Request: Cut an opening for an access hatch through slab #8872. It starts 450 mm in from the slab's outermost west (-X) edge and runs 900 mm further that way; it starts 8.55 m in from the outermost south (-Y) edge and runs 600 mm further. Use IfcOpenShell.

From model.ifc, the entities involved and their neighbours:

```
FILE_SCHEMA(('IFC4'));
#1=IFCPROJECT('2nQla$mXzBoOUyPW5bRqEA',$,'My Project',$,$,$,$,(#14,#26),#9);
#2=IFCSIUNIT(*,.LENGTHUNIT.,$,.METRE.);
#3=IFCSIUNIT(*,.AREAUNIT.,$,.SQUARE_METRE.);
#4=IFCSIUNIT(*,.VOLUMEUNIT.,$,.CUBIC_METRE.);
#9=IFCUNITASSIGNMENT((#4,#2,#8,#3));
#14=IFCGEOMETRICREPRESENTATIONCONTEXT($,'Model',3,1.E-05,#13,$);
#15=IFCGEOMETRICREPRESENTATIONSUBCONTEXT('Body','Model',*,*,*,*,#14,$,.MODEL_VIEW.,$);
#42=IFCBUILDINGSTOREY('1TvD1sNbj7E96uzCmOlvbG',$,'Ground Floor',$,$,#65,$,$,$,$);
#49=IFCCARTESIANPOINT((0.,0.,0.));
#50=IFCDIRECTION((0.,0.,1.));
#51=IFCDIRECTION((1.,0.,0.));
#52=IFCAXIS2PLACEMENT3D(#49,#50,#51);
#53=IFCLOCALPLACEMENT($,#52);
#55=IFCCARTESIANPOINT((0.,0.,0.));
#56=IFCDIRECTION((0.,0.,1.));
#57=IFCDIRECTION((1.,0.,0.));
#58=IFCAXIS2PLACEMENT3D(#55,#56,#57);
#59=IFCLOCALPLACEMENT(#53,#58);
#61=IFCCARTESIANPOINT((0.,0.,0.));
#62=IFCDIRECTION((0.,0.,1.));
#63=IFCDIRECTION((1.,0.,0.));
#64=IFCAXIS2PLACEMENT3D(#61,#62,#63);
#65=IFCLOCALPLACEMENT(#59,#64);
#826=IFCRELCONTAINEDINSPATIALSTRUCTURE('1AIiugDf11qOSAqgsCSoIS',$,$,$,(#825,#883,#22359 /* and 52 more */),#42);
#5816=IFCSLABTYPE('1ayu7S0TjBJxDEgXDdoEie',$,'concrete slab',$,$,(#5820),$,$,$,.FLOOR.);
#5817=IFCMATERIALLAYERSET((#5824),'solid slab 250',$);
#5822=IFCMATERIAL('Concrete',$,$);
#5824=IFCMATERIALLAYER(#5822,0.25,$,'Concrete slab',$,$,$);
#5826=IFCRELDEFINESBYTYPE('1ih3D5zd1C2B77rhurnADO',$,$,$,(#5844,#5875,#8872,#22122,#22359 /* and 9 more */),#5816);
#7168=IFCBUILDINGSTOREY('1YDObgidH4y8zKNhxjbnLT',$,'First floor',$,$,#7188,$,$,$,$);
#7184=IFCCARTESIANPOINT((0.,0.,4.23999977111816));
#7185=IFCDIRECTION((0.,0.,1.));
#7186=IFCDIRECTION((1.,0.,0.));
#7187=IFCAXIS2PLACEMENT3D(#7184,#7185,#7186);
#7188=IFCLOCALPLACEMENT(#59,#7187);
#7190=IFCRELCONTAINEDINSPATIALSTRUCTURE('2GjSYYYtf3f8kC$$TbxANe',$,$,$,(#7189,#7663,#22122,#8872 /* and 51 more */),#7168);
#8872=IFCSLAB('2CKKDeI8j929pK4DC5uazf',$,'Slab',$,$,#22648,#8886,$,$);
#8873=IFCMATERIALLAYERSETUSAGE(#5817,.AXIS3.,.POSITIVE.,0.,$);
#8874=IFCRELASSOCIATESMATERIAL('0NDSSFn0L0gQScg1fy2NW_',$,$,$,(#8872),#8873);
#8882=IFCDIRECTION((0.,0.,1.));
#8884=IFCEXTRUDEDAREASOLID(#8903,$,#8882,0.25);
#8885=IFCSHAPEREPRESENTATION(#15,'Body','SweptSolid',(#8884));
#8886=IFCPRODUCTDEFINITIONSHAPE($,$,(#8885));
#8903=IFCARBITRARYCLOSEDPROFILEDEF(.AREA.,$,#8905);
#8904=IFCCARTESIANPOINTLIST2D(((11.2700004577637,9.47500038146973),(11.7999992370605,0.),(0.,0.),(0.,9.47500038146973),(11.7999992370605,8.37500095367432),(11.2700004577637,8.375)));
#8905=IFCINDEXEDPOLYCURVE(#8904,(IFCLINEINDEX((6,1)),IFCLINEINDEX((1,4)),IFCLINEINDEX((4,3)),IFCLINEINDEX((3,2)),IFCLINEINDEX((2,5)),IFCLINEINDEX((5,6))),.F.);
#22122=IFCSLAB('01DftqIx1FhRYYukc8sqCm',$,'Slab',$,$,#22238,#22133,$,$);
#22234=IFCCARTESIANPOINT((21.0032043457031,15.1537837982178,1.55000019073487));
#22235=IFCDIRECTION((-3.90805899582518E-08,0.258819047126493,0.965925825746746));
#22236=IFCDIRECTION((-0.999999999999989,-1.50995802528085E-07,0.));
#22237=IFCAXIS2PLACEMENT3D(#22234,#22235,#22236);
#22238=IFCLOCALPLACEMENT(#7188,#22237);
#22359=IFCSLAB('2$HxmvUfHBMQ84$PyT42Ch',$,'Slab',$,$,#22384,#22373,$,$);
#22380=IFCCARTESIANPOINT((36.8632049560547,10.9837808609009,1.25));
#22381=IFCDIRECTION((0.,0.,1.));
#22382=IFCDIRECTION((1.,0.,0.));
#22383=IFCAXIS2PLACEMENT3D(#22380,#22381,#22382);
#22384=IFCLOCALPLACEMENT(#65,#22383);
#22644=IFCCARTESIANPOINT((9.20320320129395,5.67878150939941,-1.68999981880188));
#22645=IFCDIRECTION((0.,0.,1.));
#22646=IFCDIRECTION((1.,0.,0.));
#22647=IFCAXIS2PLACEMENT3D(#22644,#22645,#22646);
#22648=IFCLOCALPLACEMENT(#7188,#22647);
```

```python
import numpy as np
import ifcopenshell
import ifcopenshell.api.feature
import ifcopenshell.api.geometry
import ifcopenshell.api.root
import ifcopenshell.geom
import ifcopenshell.util.placement
import ifcopenshell.util.representation
import ifcopenshell.util.shape
import ifcopenshell.util.unit

model = ifcopenshell.open("model.ifc")
unit_scale = ifcopenshell.util.unit.calculate_unit_scale(model)
settings = ifcopenshell.geom.settings()


def volume(element):
    """Net volume in cubic metres, openings subtracted."""
    shape = ifcopenshell.geom.create_shape(settings, element)
    return ifcopenshell.util.shape.get_volume(shape.geometry)


slab = model.by_guid("2CKKDeI8j929pK4DC5uazf")
before = volume(slab)

# Extent in the slab's own axes, in metres. The edges named are its -X and -Y sides.
slab_shape = ifcopenshell.geom.create_shape(settings, slab)
vertices = ifcopenshell.util.shape.get_vertices(slab_shape.geometry)
x_min, y_min, bottom = vertices.min(axis=0)
top = vertices[:, 2].max()

opening = ifcopenshell.api.root.create_entity(model, ifc_class="IfcOpeningElement", name="Access hatch opening", predefined_type="OPENING")
context = ifcopenshell.util.representation.get_context(model, "Model", "Body", "MODEL_VIEW")
width, depth = 0.9, 0.6
outline = [(0.0, 0.0), (width, 0.0), (width, depth), (0.0, depth), (0.0, 0.0)]
# Overshoot both faces by 50 mm so the cut is clean.
shape = ifcopenshell.api.geometry.add_slab_representation(
    model, context=context, depth=top - bottom + 0.1, polyline=outline
)
ifcopenshell.api.geometry.assign_representation(model, product=opening, representation=shape)

matrix = ifcopenshell.util.placement.get_local_placement(slab.ObjectPlacement)
matrix[:, 3] = matrix @ np.append(np.array([x_min + 0.45, y_min + 8.55, bottom - 0.05]) / unit_scale, 1.0)
ifcopenshell.api.geometry.edit_object_placement(model, product=opening, matrix=matrix, is_si=False)
ifcopenshell.api.feature.add_feature(model, feature=opening, element=slab)

after = volume(slab)

print(f"slab volume {before:.3f} -> {after:.3f} m3")

model.write("model-out.ifc")
```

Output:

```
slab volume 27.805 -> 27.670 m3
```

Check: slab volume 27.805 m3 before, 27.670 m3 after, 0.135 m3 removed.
